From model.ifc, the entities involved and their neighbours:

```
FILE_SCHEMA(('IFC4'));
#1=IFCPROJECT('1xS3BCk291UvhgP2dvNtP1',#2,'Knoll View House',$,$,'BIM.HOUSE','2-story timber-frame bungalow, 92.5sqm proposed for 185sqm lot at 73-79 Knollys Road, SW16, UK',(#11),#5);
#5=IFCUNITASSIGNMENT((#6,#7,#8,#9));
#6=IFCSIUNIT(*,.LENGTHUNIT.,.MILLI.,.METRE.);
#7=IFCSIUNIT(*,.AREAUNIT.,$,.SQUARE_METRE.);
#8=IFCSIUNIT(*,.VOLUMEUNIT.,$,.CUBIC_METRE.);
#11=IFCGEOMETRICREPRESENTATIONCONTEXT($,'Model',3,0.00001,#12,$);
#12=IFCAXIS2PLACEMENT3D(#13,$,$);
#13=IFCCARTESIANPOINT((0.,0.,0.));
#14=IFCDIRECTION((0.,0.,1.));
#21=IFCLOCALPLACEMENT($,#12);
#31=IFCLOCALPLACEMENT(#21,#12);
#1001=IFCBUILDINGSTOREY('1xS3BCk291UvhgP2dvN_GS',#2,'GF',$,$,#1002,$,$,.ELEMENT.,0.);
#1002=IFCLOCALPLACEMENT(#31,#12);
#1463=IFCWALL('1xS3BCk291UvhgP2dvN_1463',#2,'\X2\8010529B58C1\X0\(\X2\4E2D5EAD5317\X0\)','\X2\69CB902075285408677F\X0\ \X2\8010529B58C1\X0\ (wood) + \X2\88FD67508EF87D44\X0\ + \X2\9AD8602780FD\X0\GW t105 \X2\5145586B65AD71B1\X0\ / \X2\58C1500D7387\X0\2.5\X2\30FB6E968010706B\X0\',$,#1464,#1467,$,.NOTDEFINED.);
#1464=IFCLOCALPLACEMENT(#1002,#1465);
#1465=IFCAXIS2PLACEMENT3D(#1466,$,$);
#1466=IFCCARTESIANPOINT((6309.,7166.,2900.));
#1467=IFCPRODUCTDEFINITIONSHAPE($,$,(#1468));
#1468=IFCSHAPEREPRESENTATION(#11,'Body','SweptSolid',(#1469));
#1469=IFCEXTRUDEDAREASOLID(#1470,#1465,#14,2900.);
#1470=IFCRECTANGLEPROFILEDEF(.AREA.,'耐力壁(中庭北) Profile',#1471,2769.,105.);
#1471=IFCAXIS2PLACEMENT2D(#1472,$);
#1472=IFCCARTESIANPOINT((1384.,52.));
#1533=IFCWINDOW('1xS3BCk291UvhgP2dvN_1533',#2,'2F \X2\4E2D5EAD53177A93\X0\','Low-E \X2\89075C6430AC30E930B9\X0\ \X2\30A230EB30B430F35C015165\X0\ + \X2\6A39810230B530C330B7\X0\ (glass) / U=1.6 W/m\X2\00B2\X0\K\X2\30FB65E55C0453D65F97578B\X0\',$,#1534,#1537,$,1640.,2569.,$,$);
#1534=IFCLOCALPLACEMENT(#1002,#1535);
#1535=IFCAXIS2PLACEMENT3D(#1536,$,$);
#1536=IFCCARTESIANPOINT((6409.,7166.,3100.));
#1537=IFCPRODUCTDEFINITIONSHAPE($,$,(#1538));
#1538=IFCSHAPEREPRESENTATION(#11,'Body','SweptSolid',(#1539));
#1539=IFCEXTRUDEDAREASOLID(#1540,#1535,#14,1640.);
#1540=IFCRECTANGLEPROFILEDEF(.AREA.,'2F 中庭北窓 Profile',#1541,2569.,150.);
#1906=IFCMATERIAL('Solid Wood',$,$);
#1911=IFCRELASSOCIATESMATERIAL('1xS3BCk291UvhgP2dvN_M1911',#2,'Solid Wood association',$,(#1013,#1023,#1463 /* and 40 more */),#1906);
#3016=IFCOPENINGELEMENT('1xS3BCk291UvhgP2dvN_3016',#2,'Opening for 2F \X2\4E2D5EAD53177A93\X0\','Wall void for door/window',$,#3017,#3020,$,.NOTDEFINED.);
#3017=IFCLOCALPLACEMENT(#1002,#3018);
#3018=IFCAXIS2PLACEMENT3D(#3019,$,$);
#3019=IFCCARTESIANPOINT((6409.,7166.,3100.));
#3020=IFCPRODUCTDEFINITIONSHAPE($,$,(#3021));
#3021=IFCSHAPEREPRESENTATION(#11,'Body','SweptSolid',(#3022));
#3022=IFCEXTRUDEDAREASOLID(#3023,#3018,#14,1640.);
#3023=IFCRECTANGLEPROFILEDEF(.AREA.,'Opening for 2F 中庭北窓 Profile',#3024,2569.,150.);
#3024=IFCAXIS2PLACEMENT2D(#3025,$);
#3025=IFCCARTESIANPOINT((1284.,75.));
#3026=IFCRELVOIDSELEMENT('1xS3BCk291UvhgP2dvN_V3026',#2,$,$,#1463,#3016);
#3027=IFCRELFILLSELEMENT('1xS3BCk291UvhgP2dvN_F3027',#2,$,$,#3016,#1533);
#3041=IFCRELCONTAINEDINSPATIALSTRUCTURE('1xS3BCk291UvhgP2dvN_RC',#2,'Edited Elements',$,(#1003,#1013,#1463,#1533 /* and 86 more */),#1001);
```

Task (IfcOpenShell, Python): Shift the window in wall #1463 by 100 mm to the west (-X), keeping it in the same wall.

```python
import ifcopenshell
import ifcopenshell.api.geometry
import ifcopenshell.util.placement
import ifcopenshell.util.unit

model = ifcopenshell.open("model.ifc")
unit_scale = ifcopenshell.util.unit.calculate_unit_scale(model)

window = model.by_id(1533)
opening = window.FillsVoids[0].RelatingOpeningElement
wall = opening.VoidsElements[0].RelatingBuildingElement

wall_matrix = ifcopenshell.util.placement.get_local_placement(wall.ObjectPlacement)
shift = wall_matrix[:3, 0] * -0.1 / unit_scale
before = ifcopenshell.util.placement.get_local_placement(window.ObjectPlacement)[:3, 3].copy()

# The window is not placed relative to its opening, so move both.
for product in (opening, window):
    matrix = ifcopenshell.util.placement.get_local_placement(product.ObjectPlacement)
    matrix[:3, 3] += shift
    ifcopenshell.api.geometry.edit_object_placement(model, product=product, matrix=matrix, is_si=False)

after = ifcopenshell.util.placement.get_local_placement(window.ObjectPlacement)[:3, 3]
print("window moved by", (after - before).round(3) + 0.0)

model.write("model_updated.ifc")
```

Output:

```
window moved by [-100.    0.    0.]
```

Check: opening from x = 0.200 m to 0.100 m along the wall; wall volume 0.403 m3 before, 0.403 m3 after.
